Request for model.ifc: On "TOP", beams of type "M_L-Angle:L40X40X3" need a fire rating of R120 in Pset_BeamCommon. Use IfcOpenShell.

First a look at what the model holds.

```python
import ifcopenshell
import ifcopenshell.util.element

model = ifcopenshell.open("model.ifc")
print(model.schema)
storey = next(s for s in model.by_type("IfcBuildingStorey") if s.Name == "TOP")
beams = [e for e in ifcopenshell.util.element.get_decomposition(storey) if e.is_a("IfcBeam")]
seen = {}
for e in beams:
    element_type = ifcopenshell.util.element.get_type(e)
    key = (element_type.Name if element_type != e and element_type else None, ifcopenshell.util.element.get_pset(e, "Pset_BeamCommon", "FireRating"))
    seen[key] = seen.get(key, 0) + 1
for (name, value), count in sorted(seen.items(), key=str):
    print(count, "x", name, "|", value)
```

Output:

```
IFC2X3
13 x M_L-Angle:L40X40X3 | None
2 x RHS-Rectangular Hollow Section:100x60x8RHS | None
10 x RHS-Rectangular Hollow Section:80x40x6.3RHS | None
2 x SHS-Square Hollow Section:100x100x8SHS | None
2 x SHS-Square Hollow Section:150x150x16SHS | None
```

```python
import ifcopenshell
import ifcopenshell.api.pset
import ifcopenshell.util.element

model = ifcopenshell.open("model.ifc")

storey = next(s for s in model.by_type("IfcBuildingStorey") if s.Name == "TOP")
beams = [e for e in ifcopenshell.util.element.get_decomposition(storey) if e.is_a("IfcBeam")]

count = 0
for e in beams:
    element_type = ifcopenshell.util.element.get_type(e)
    if element_type in (None, e) or element_type.Name != "M_L-Angle:L40X40X3":
        continue
    # add_pset returns the element's existing set when there is one.
    pset = ifcopenshell.api.pset.add_pset(model, product=e, name="Pset_BeamCommon")
    ifcopenshell.api.pset.edit_pset(model, pset=pset, properties={"FireRating": "R120"})
    count += 1

print(count, "beams updated")

model.write("model_updated.ifc")
```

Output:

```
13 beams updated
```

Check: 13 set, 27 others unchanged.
